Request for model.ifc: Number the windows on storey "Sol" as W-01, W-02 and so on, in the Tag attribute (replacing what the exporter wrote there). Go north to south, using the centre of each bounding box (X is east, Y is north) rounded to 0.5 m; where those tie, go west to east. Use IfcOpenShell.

First a look at what the model holds.

```python
import ifcopenshell
import ifcopenshell.util.element
import ifcopenshell.util.placement

model = ifcopenshell.open("model.ifc")
print(model.schema)
storey = next(s for s in model.by_type("IfcBuildingStorey") if s.Name == "Sol")
windows = [e for e in ifcopenshell.util.element.get_decomposition(storey) if e.is_a("IfcWindow")]
for e in sorted(windows, key=lambda e: e.id()):
    origin = ifcopenshell.util.placement.get_local_placement(e.ObjectPlacement)[:3, 3]
    print(e.id(), e.Tag, e.Name, origin.round(2) + 0.0, sep=" | ")
```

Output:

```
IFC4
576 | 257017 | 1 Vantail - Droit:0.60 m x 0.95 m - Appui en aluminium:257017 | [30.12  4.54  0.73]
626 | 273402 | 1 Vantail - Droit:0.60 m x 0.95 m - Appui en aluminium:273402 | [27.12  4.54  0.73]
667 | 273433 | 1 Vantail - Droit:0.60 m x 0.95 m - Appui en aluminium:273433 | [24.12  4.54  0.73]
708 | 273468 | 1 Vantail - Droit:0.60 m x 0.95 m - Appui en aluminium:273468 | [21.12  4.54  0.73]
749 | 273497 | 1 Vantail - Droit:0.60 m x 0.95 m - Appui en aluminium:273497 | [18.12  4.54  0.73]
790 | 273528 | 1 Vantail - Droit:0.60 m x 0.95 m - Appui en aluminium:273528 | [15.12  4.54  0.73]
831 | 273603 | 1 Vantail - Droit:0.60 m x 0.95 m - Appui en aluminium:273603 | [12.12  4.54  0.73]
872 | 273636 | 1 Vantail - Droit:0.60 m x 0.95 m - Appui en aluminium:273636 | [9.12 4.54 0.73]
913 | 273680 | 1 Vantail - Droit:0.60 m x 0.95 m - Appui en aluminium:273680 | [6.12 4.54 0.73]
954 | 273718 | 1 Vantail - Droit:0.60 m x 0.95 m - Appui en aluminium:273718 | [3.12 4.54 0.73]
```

```python
import ifcopenshell
import ifcopenshell.geom
import ifcopenshell.util.element
import ifcopenshell.util.shape

model = ifcopenshell.open("model.ifc")
settings = ifcopenshell.geom.settings()
settings.set("use-world-coords", True)


def centre(element):
    shape = ifcopenshell.geom.create_shape(settings, element)
    return ifcopenshell.util.shape.get_bbox_centroid(shape.geometry)


storey = next(s for s in model.by_type("IfcBuildingStorey") if s.Name == "Sol")
windows = [e for e in ifcopenshell.util.element.get_decomposition(storey) if e.is_a("IfcWindow")]

# Insertion points can sit at a corner or the storey origin, so sort by the geometry (in metres).
centres = {e: centre(e) for e in windows}
windows.sort(key=lambda e: (-round(centres[e][1] / 0.5), centres[e][0]))

for i, e in enumerate(windows, start=1):
    number = f"W-{i:02d}"
    e.Tag = number
    print(e.id(), number)

model.write("model_v2.ifc")
```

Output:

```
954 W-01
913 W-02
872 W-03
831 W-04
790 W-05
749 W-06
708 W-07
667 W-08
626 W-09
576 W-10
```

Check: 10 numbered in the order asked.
